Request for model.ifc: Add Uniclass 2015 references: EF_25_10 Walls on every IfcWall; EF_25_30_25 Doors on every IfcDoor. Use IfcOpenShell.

First a look at what the model holds.

```python
import ifcopenshell

model = ifcopenshell.open("model.ifc")
print(model.schema)
print("classifications:", [c.Name for c in model.by_type("IfcClassification")])
for ifc_class in ("IfcDoor", "IfcRoof", "IfcStair", "IfcWall", "IfcWindow"):
    print(ifc_class, len(model.by_type(ifc_class)))
```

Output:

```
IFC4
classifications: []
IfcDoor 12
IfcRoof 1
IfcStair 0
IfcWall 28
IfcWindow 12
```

```python
import ifcopenshell
import ifcopenshell.api.classification

model = ifcopenshell.open("model.ifc")

system = ifcopenshell.api.classification.add_classification(model, classification="Uniclass 2015")

codes = {
    "IfcWall": ("EF_25_10", "Walls"),
    "IfcDoor": ("EF_25_30_25", "Doors"),
}
for ifc_class, (code, name) in codes.items():
    products = model.by_type(ifc_class)
    ifcopenshell.api.classification.add_reference(
        model, products=products, classification=system, identification=code, name=name
    )
    print(code, len(products))

model.write("model_rev.ifc")
```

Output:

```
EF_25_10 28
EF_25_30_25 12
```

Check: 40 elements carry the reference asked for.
